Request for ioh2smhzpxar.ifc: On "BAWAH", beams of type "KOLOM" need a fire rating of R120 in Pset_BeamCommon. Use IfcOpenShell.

First a look at what the model holds.

```python
import ifcopenshell
import ifcopenshell.util.element

model = ifcopenshell.open("ioh2smhzpxar.ifc")
print(model.schema)
storey = next(s for s in model.by_type("IfcBuildingStorey") if s.Name == "BAWAH")
beams = [e for e in ifcopenshell.util.element.get_decomposition(storey) if e.is_a("IfcBeam")]
seen = {}
for e in beams:
    element_type = ifcopenshell.util.element.get_type(e)
    key = (element_type.Name if element_type != e and element_type else None, ifcopenshell.util.element.get_pset(e, "Pset_BeamCommon", "FireRating"))
    seen[key] = seen.get(key, 0) + 1
for (name, value), count in sorted(seen.items(), key=str):
    print(count, "x", name, "|", value)
```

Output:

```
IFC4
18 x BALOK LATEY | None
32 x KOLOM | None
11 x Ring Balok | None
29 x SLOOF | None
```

```python
import ifcopenshell
import ifcopenshell.api.pset
import ifcopenshell.util.element

model = ifcopenshell.open("ioh2smhzpxar.ifc")

storey = next(s for s in model.by_type("IfcBuildingStorey") if s.Name == "BAWAH")
beams = [e for e in ifcopenshell.util.element.get_decomposition(storey) if e.is_a("IfcBeam")]

count = 0
for e in beams:
    element_type = ifcopenshell.util.element.get_type(e)
    if element_type in (None, e) or element_type.Name != "KOLOM":
        continue
    # add_pset returns the element's existing set when there is one.
    pset = ifcopenshell.api.pset.add_pset(model, product=e, name="Pset_BeamCommon")
    ifcopenshell.api.pset.edit_pset(model, pset=pset, properties={"FireRating": "R120"})
    count += 1

print(count, "beams updated")

model.write("ioh2smhzpxar_updated.ifc")
```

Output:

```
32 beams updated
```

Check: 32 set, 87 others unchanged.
